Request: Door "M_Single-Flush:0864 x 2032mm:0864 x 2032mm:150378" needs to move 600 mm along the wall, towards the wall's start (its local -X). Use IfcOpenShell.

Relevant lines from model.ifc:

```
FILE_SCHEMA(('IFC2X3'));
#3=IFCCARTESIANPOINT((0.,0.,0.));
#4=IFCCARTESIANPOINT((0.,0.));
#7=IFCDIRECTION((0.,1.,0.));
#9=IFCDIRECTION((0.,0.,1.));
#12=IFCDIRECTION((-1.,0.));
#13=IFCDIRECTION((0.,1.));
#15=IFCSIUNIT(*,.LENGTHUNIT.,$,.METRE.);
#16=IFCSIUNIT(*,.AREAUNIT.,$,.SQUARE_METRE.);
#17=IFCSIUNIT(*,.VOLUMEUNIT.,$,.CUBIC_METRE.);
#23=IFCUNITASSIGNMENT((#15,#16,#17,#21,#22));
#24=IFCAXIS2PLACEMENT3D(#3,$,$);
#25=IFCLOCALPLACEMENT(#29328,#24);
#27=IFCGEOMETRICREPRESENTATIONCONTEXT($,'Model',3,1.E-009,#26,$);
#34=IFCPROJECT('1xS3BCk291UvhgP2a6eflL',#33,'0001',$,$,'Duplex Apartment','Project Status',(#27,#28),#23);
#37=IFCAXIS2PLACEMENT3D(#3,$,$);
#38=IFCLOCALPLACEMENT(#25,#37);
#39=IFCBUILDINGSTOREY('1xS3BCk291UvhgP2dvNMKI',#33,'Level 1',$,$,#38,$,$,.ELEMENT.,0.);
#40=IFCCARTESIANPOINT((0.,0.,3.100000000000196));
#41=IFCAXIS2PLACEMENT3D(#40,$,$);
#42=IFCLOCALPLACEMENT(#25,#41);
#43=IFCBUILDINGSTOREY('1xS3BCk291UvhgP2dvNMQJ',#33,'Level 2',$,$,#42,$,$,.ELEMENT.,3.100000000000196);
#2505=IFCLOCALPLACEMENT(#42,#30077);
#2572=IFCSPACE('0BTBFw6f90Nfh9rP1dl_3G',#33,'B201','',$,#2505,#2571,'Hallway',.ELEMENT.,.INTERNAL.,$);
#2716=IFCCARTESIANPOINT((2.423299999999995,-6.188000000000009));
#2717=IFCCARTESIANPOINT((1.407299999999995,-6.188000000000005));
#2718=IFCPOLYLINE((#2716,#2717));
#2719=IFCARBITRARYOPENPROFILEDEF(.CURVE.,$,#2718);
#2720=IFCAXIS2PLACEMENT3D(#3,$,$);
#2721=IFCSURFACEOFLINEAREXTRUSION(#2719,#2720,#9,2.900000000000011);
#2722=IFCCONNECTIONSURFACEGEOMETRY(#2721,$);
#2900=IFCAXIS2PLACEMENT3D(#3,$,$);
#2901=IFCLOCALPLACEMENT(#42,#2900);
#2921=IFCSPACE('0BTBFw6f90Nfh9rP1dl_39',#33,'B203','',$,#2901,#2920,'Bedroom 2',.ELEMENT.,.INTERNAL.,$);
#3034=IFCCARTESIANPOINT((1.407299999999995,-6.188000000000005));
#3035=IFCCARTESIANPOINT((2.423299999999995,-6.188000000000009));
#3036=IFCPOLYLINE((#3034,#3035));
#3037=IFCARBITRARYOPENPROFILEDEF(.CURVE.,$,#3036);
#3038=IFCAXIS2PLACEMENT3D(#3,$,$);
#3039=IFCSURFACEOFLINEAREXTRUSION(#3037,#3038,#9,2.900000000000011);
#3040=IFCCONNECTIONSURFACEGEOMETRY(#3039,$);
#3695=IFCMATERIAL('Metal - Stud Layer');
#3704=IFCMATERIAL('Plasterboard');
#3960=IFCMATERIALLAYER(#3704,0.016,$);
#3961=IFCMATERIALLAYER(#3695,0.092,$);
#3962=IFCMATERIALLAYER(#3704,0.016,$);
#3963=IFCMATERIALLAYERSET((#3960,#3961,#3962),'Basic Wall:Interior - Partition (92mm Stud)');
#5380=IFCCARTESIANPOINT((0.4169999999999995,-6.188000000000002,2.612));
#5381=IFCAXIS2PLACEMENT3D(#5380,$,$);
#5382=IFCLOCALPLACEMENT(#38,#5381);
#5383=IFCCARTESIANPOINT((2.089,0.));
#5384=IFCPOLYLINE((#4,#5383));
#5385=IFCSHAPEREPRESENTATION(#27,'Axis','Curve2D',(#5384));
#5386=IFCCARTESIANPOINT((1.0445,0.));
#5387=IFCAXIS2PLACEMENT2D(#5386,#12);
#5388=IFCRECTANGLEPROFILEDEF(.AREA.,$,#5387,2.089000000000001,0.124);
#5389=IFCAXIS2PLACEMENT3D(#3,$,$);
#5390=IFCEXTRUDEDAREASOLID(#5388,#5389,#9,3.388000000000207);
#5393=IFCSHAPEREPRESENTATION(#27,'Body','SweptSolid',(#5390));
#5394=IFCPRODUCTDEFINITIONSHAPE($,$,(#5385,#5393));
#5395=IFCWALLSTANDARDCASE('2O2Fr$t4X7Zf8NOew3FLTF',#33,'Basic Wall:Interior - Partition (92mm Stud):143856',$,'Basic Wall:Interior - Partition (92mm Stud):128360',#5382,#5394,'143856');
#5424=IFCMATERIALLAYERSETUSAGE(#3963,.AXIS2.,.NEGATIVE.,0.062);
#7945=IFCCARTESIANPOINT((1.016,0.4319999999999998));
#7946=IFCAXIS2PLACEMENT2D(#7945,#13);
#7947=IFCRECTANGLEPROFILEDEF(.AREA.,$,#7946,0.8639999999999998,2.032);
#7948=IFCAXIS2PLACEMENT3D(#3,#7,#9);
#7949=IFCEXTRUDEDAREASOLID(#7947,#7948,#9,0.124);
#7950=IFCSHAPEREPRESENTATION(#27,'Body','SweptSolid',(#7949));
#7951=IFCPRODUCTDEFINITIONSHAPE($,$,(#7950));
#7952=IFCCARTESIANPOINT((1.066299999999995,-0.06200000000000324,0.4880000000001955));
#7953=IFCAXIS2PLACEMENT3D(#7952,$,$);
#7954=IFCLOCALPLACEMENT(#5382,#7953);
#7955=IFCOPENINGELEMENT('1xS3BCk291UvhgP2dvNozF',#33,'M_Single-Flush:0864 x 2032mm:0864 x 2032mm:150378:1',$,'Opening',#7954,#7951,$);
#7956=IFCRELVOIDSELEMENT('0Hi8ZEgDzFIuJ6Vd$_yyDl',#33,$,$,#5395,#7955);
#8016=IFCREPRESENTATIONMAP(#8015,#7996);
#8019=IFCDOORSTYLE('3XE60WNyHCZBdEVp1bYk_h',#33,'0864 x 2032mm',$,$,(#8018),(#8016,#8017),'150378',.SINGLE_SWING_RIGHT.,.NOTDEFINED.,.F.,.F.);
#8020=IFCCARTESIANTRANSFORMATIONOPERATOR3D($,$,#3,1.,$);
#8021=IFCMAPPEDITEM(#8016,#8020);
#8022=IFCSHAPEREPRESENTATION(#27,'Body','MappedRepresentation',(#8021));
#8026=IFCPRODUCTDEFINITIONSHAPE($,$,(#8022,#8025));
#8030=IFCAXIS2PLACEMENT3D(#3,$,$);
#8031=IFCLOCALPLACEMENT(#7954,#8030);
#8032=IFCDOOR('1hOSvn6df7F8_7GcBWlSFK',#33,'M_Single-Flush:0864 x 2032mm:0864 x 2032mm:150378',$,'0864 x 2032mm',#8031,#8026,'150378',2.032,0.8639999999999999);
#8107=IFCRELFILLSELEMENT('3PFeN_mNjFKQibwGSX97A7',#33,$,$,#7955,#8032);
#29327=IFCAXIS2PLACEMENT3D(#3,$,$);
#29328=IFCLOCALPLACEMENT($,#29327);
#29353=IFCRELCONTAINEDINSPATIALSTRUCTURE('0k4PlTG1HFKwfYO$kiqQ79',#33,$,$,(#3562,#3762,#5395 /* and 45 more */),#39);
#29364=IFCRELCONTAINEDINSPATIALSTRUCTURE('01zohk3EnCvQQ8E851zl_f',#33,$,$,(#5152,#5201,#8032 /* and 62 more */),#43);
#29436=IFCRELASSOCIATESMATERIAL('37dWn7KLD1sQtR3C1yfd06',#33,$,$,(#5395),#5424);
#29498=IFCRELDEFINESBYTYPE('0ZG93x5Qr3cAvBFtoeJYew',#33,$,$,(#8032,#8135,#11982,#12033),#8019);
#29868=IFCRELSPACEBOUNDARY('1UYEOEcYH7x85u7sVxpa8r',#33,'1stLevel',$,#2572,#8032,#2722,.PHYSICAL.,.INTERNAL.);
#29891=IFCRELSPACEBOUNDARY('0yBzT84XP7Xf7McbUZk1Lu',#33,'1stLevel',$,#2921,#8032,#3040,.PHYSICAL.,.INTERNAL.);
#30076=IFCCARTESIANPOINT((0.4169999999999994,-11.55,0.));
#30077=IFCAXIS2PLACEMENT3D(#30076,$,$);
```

```python
import numpy as np
import ifcopenshell
import ifcopenshell.api.geometry
import ifcopenshell.util.placement

model = ifcopenshell.open("model.ifc")

door = model.by_id(8032)
opening = door.FillsVoids[0].RelatingOpeningElement
wall = opening.VoidsElements[0].RelatingBuildingElement

wall_matrix = ifcopenshell.util.placement.get_local_placement(wall.ObjectPlacement)
shift = wall_matrix[:3, 0] * -0.6
before = ifcopenshell.util.placement.get_local_placement(door.ObjectPlacement)[:3, 3].copy()

# The door is placed relative to its opening, so it follows when the opening moves.
matrix = ifcopenshell.util.placement.get_local_placement(opening.ObjectPlacement)
matrix[:3, 3] += shift
ifcopenshell.api.geometry.edit_object_placement(
    model, product=opening, matrix=matrix, is_si=False, should_transform_children=True
)

# Space boundary surfaces are stored in each space's coordinates; move them too.
for rel in door.ProvidesBoundaries:
    if not rel.ConnectionGeometry:
        continue
    surface = rel.ConnectionGeometry.SurfaceOnRelatingElement
    space_matrix = ifcopenshell.util.placement.get_local_placement(rel.RelatingSpace.ObjectPlacement)
    point = np.array(surface.Position.Location.Coordinates) + space_matrix[:3, :3].T @ shift
    surface.Position = model.createIfcAxis2Placement3D(
        model.createIfcCartesianPoint(point.tolist()), surface.Position.Axis, surface.Position.RefDirection
    )

after = ifcopenshell.util.placement.get_local_placement(door.ObjectPlacement)[:3, 3]
print("door moved by", (after - before).round(3) + 0.0)

model.write("model_rev.ifc")
```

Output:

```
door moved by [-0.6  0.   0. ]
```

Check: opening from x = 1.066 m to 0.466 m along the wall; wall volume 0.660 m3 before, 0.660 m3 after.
